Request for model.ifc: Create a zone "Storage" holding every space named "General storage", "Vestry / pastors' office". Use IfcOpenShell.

First a look at what the model holds.

```python
import ifcopenshell

model = ifcopenshell.open("model.ifc")
print(model.schema)
seen = {}
for space in model.by_type("IfcSpace"):
    seen[space.LongName] = seen.get(space.LongName, 0) + 1
for name, count in sorted(seen.items(), key=str):
    print(count, "x", name)
print("zones:", [z.Name for z in model.by_type("IfcZone")][:20])
```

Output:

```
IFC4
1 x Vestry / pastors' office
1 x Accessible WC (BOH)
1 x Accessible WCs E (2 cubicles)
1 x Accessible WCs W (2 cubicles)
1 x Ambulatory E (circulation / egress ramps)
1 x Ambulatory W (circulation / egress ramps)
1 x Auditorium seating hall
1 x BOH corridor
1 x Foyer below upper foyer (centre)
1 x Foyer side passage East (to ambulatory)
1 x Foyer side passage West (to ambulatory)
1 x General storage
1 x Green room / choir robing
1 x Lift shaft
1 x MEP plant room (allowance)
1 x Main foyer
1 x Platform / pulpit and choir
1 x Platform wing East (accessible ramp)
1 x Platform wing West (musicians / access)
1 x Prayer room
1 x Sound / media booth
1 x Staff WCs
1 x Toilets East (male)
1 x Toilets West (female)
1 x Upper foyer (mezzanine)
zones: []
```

```python
import ifcopenshell
import ifcopenshell.api.group
import ifcopenshell.api.root

model = ifcopenshell.open("model.ifc")

names = {"General storage", "Vestry / pastors' office"}
spaces = [s for s in model.by_type("IfcSpace") if s.LongName in names]

zone = ifcopenshell.api.root.create_entity(model, ifc_class="IfcZone", name="Storage")
ifcopenshell.api.group.assign_group(model, products=spaces, group=zone)
print(len(spaces), "spaces in", zone.Name)

model.write("model_edited.ifc")
```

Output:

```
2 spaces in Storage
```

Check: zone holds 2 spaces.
